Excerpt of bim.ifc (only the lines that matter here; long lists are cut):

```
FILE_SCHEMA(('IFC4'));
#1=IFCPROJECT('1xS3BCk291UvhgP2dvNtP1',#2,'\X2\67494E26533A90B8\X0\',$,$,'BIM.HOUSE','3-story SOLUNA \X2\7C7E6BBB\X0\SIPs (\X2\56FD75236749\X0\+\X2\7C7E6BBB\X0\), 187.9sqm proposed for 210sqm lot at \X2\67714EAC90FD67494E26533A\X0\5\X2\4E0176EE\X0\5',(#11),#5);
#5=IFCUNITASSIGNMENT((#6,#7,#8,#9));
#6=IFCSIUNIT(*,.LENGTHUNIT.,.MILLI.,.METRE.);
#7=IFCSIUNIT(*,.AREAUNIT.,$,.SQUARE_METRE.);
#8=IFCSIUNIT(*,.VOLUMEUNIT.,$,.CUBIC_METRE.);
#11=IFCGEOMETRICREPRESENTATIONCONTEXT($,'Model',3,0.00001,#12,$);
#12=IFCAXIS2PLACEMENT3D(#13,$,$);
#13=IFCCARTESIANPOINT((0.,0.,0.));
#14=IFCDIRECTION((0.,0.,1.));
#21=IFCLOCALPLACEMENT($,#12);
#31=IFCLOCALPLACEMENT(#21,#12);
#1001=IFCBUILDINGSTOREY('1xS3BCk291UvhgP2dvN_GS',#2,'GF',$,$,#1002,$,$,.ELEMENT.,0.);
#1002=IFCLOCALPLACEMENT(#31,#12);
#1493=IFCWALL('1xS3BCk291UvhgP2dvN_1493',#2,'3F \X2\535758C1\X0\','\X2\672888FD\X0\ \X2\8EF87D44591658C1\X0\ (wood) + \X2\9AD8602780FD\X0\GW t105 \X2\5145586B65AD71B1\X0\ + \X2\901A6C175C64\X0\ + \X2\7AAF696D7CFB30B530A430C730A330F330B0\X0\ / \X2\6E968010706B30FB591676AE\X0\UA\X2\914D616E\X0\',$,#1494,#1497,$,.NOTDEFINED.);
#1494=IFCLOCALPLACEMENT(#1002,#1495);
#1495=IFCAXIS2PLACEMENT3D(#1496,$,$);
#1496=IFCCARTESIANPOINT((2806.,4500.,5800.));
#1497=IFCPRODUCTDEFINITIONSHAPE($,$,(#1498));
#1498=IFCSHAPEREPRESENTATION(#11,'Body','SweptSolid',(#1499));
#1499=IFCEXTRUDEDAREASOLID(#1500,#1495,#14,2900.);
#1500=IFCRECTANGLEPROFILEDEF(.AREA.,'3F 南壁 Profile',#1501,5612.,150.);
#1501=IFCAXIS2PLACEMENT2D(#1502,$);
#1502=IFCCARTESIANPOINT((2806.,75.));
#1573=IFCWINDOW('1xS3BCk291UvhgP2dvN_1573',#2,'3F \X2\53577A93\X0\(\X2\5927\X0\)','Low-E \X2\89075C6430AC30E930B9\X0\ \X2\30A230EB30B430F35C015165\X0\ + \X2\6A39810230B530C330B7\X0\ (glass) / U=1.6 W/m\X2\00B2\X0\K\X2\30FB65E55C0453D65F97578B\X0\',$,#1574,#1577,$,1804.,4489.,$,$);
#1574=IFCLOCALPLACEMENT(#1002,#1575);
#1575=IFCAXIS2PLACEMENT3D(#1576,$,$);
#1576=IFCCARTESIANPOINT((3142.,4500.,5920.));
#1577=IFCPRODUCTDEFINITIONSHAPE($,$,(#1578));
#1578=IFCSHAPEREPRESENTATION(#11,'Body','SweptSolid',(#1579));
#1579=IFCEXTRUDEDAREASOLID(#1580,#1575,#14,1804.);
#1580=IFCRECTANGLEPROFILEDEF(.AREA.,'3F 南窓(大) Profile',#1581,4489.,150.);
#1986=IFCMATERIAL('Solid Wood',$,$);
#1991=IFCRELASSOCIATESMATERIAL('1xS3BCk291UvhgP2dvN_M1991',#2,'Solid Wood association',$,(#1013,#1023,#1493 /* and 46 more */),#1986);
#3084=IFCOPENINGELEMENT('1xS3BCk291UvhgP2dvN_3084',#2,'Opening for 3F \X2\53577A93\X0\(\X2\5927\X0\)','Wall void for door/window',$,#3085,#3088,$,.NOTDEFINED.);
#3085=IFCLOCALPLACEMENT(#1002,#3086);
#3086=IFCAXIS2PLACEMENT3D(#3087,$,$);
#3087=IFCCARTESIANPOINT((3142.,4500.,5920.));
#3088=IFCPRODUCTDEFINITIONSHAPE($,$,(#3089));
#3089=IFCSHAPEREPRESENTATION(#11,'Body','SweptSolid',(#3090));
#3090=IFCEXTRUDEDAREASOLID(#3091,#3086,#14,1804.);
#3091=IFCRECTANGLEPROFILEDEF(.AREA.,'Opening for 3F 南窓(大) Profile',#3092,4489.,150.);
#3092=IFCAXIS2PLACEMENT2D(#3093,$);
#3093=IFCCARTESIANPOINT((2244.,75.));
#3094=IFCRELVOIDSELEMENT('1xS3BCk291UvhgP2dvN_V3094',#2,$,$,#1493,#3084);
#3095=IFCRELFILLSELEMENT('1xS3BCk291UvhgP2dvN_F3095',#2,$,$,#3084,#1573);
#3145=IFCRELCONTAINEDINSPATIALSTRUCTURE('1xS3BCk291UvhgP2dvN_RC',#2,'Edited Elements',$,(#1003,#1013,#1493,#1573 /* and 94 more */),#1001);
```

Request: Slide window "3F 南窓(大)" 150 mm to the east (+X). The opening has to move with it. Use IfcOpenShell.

```python
import ifcopenshell
import ifcopenshell.api.geometry
import ifcopenshell.util.placement

model = ifcopenshell.open("bim.ifc")

window = model.by_guid("1xS3BCk291UvhgP2dvN_1573")
opening = window.FillsVoids[0].RelatingOpeningElement
wall = opening.VoidsElements[0].RelatingBuildingElement

wall_matrix = ifcopenshell.util.placement.get_local_placement(wall.ObjectPlacement)
shift = wall_matrix[:3, 0] * 150.0
before = ifcopenshell.util.placement.get_local_placement(window.ObjectPlacement)[:3, 3].copy()

# The window is not placed relative to its opening, so move both.
for product in (opening, window):
    matrix = ifcopenshell.util.placement.get_local_placement(product.ObjectPlacement)
    matrix[:3, 3] += shift
    ifcopenshell.api.geometry.edit_object_placement(model, product=product, matrix=matrix, is_si=False)

after = ifcopenshell.util.placement.get_local_placement(window.ObjectPlacement)[:3, 3]
print("window moved by", (after - before).round(3) + 0.0)

model.write("bim_updated.ifc")
```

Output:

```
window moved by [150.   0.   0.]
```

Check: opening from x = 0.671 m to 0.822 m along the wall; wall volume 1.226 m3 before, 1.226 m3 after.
